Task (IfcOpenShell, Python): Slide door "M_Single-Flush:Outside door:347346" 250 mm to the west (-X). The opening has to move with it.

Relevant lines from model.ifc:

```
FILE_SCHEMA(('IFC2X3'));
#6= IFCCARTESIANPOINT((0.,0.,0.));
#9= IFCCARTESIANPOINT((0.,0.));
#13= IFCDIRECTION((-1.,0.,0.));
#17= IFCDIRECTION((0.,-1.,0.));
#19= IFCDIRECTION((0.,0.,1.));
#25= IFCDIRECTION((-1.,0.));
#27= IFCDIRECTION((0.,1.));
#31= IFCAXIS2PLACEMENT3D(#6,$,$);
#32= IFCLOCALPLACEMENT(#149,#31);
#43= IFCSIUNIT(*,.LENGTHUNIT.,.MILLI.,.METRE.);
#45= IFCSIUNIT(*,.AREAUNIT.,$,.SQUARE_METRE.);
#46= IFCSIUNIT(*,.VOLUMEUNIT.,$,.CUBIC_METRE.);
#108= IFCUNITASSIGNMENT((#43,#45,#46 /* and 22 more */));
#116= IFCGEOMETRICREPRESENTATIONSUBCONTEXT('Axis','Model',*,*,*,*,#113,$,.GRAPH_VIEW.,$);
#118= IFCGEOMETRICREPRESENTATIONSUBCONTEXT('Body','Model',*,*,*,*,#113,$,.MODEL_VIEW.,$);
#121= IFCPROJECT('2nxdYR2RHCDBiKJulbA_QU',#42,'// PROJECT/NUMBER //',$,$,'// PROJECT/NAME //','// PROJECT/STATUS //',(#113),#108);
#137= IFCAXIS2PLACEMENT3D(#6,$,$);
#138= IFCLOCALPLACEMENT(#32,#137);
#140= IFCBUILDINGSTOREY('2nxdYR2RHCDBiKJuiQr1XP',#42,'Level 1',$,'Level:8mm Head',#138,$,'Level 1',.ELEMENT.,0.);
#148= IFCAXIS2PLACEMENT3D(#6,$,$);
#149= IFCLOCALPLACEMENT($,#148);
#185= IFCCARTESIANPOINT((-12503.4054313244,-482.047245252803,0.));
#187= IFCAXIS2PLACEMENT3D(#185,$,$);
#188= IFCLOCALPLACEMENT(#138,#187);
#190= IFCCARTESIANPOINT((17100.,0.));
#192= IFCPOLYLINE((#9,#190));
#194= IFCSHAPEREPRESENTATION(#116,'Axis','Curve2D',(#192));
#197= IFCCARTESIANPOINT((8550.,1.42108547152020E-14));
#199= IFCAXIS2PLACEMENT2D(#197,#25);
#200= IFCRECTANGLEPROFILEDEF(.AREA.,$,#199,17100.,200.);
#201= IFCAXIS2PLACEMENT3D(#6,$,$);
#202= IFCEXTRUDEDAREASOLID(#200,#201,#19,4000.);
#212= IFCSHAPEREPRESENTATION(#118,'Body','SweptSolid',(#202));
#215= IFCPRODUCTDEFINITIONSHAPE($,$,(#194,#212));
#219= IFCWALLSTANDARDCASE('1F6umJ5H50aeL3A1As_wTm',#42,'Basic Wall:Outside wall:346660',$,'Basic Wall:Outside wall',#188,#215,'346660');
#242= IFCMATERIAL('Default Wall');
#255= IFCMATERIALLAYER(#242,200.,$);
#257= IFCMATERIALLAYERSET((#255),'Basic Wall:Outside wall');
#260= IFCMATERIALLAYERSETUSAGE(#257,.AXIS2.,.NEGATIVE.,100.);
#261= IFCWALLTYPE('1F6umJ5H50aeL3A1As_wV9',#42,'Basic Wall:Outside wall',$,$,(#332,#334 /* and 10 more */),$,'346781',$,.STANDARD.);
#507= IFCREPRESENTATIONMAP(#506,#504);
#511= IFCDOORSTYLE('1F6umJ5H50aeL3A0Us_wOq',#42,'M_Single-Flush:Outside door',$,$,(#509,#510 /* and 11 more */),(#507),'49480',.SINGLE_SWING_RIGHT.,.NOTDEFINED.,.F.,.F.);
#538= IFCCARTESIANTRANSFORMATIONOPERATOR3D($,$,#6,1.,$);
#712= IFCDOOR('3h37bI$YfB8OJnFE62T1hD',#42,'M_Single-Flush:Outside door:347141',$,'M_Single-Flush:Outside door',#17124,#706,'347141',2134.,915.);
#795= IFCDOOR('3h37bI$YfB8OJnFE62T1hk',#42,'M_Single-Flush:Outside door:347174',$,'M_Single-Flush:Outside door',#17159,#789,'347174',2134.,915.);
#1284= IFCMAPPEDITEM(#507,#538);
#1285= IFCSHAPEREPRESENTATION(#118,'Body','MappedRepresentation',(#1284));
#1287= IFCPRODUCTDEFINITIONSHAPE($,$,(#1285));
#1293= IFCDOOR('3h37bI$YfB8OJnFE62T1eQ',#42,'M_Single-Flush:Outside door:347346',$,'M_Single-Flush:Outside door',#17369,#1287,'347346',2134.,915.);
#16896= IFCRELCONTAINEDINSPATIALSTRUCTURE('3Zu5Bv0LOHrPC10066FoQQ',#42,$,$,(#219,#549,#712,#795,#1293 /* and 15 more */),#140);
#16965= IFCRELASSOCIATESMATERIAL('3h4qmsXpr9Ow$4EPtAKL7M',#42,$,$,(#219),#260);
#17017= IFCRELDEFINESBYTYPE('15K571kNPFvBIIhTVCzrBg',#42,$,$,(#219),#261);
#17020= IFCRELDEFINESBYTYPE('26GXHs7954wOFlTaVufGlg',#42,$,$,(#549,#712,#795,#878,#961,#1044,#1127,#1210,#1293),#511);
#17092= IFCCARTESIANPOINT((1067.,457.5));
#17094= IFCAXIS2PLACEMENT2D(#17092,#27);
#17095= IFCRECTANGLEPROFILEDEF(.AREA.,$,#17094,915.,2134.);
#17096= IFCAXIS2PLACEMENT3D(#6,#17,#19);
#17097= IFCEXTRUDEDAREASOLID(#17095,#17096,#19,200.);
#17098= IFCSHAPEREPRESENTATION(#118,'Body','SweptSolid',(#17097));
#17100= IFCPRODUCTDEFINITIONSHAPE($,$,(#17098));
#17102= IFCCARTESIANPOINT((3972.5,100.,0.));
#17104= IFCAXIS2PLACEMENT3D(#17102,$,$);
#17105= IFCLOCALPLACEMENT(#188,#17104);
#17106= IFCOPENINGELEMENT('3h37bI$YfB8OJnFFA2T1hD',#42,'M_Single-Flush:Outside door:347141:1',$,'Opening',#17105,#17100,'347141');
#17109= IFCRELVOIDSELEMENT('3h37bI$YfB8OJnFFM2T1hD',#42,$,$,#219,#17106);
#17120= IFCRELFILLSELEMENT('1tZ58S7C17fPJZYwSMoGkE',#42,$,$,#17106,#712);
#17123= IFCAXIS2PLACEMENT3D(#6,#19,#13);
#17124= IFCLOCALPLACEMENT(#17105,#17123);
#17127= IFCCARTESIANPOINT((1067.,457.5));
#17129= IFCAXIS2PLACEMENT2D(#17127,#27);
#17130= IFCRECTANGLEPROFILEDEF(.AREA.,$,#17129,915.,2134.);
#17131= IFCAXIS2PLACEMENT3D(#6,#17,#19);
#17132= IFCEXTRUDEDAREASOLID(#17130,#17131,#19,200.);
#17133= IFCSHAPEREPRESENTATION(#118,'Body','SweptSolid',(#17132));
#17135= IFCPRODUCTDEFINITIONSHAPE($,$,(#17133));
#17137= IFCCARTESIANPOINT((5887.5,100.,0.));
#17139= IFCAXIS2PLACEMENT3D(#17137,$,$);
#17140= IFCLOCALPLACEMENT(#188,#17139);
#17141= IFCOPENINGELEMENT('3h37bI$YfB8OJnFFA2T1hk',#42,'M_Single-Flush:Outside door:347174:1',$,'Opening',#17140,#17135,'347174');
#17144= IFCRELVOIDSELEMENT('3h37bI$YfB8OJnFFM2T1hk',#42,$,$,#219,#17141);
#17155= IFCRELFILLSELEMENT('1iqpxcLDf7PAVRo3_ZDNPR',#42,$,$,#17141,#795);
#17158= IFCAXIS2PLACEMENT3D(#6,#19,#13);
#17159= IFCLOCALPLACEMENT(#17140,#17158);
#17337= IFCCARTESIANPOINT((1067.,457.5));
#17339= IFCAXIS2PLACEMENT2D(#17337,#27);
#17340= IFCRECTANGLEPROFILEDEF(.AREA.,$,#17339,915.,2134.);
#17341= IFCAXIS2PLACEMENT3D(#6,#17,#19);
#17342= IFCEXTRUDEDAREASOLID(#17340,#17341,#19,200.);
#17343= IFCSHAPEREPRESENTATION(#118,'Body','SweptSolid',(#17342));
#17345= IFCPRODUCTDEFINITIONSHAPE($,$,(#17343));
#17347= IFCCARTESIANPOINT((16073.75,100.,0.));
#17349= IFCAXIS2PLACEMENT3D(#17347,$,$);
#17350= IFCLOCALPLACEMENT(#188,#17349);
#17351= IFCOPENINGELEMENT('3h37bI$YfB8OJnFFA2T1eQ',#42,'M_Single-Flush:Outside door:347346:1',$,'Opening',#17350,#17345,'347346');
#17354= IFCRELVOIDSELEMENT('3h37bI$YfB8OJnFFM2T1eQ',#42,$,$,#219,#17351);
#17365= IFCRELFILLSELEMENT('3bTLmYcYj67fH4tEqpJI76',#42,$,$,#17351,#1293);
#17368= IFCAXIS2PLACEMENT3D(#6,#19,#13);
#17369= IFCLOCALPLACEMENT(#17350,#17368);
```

```python
import ifcopenshell
import ifcopenshell.api.geometry
import ifcopenshell.util.placement
import ifcopenshell.util.unit

model = ifcopenshell.open("model.ifc")
unit_scale = ifcopenshell.util.unit.calculate_unit_scale(model)

door = model.by_guid("3h37bI$YfB8OJnFE62T1eQ")
opening = door.FillsVoids[0].RelatingOpeningElement
wall = opening.VoidsElements[0].RelatingBuildingElement

wall_matrix = ifcopenshell.util.placement.get_local_placement(wall.ObjectPlacement)
shift = wall_matrix[:3, 0] * -0.25 / unit_scale
before = ifcopenshell.util.placement.get_local_placement(door.ObjectPlacement)[:3, 3].copy()

# The door is placed relative to its opening, so it follows when the opening moves.
matrix = ifcopenshell.util.placement.get_local_placement(opening.ObjectPlacement)
matrix[:3, 3] += shift
ifcopenshell.api.geometry.edit_object_placement(
    model, product=opening, matrix=matrix, is_si=False, should_transform_children=True
)

after = ifcopenshell.util.placement.get_local_placement(door.ObjectPlacement)[:3, 3]
print("door moved by", (after - before).round(3) + 0.0)

model.write("model_edited.ifc")
```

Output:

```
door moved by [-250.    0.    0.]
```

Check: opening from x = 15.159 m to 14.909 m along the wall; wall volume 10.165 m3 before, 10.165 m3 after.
